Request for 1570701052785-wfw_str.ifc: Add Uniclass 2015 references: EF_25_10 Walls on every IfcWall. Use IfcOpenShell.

First a look at what the model holds.

```python
import ifcopenshell

model = ifcopenshell.open("1570701052785-wfw_str.ifc")
print(model.schema)
print("classifications:", [c.Name for c in model.by_type("IfcClassification")])
for ifc_class in ("IfcDoor", "IfcRoof", "IfcStair", "IfcWall", "IfcWindow"):
    print(ifc_class, len(model.by_type(ifc_class)))
```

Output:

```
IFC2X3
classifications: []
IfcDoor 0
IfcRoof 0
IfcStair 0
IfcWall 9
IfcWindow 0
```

```python
import ifcopenshell
import ifcopenshell.api.classification

model = ifcopenshell.open("1570701052785-wfw_str.ifc")

# IFC2X3 requires Source and Edition and has no link from the project to the system.
system = model.create_entity("IfcClassification", Source="NBS", Edition="2015", Name="Uniclass 2015")

codes = {
    "IfcWall": ("EF_25_10", "Walls"),
}
for ifc_class, (code, name) in codes.items():
    products = model.by_type(ifc_class)
    ifcopenshell.api.classification.add_reference(
        model, products=products, classification=system, identification=code, name=name
    )
    print(code, len(products))

model.write("1570701052785-wfw_str_v2.ifc")
```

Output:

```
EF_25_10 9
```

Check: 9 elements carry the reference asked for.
